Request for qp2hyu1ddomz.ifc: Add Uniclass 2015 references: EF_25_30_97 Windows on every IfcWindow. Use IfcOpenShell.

First a look at what the model holds.

```python
import ifcopenshell

model = ifcopenshell.open("qp2hyu1ddomz.ifc")
print(model.schema)
print("classifications:", [c.Name for c in model.by_type("IfcClassification")])
for ifc_class in ("IfcDoor", "IfcRoof", "IfcStair", "IfcWall", "IfcWindow"):
    print(ifc_class, len(model.by_type(ifc_class)))
```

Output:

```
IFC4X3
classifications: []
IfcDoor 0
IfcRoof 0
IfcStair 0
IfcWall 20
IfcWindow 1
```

```python
import ifcopenshell
import ifcopenshell.api.classification

model = ifcopenshell.open("qp2hyu1ddomz.ifc")

system = ifcopenshell.api.classification.add_classification(model, classification="Uniclass 2015")

codes = {
    "IfcWindow": ("EF_25_30_97", "Windows"),
}
for ifc_class, (code, name) in codes.items():
    products = model.by_type(ifc_class)
    ifcopenshell.api.classification.add_reference(
        model, products=products, classification=system, identification=code, name=name
    )
    print(code, len(products))

model.write("qp2hyu1ddomz_edited.ifc")
```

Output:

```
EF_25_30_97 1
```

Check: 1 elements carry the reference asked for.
